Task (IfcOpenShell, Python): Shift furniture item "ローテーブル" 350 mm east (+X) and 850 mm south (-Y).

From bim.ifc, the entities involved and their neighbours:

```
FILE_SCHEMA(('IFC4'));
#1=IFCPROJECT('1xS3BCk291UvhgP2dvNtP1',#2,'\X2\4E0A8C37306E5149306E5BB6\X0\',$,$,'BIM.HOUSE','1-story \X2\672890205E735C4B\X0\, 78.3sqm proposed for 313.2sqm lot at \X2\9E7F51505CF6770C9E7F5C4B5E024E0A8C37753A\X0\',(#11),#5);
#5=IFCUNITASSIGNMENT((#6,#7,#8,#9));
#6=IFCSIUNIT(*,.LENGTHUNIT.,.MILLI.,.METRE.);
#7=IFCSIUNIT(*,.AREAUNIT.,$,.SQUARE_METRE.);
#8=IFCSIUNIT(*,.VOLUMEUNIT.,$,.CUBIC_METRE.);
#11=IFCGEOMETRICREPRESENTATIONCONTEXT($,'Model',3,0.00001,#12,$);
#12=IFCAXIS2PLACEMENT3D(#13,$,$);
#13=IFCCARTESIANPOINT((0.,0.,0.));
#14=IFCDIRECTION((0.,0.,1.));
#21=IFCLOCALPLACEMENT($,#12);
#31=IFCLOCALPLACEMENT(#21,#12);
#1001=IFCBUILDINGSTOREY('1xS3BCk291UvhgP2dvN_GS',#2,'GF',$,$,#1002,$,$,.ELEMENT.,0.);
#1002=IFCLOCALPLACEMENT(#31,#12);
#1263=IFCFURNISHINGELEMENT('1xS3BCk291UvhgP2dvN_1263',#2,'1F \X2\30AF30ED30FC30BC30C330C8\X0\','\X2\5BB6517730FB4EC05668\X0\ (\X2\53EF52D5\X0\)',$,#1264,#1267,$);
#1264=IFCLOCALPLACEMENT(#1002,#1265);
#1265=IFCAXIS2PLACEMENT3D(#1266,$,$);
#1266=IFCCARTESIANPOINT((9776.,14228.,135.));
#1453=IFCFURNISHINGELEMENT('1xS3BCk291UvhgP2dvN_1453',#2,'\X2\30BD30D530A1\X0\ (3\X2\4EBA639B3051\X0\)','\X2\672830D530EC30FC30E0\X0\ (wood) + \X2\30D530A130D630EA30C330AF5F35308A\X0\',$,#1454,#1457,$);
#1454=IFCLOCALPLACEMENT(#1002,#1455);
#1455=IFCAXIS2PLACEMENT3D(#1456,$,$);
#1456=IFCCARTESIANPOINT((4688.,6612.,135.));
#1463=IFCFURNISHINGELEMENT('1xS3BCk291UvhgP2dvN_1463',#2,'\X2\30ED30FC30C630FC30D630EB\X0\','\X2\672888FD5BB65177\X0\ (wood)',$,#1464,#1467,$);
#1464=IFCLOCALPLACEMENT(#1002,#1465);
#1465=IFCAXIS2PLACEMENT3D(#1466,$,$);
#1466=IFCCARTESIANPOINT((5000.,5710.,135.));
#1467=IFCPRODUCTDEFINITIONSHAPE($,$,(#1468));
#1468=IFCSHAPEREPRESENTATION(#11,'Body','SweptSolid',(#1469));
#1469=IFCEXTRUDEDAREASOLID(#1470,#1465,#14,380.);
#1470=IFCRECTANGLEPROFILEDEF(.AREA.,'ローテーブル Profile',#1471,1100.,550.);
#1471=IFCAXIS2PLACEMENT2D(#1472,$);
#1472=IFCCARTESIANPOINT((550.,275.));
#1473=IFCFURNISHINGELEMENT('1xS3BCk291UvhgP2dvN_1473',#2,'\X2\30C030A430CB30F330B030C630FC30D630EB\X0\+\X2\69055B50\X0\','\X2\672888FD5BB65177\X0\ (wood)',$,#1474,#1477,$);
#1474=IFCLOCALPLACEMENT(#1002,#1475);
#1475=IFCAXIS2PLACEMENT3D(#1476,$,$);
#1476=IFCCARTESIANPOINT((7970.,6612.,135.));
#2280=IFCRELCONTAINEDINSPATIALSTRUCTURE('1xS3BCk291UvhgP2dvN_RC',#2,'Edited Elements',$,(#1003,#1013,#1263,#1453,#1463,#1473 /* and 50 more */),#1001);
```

```python
import ifcopenshell
import ifcopenshell.api.geometry
import ifcopenshell.util.placement
import ifcopenshell.util.unit

model = ifcopenshell.open("bim.ifc")
unit_scale = ifcopenshell.util.unit.calculate_unit_scale(model)

item = model.by_guid("1xS3BCk291UvhgP2dvN_1463")
matrix = ifcopenshell.util.placement.get_local_placement(item.ObjectPlacement)
matrix[0, 3] += 0.35 / unit_scale
matrix[1, 3] -= 0.85 / unit_scale
ifcopenshell.api.geometry.edit_object_placement(model, product=item, matrix=matrix, is_si=False)

print(ifcopenshell.util.placement.get_local_placement(item.ObjectPlacement).round(3) + 0.0)

model.write("bim_updated.ifc")
```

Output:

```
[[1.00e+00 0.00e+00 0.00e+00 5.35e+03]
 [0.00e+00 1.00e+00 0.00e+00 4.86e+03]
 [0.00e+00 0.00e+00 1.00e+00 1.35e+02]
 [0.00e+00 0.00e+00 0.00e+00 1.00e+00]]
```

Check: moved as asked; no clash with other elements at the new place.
